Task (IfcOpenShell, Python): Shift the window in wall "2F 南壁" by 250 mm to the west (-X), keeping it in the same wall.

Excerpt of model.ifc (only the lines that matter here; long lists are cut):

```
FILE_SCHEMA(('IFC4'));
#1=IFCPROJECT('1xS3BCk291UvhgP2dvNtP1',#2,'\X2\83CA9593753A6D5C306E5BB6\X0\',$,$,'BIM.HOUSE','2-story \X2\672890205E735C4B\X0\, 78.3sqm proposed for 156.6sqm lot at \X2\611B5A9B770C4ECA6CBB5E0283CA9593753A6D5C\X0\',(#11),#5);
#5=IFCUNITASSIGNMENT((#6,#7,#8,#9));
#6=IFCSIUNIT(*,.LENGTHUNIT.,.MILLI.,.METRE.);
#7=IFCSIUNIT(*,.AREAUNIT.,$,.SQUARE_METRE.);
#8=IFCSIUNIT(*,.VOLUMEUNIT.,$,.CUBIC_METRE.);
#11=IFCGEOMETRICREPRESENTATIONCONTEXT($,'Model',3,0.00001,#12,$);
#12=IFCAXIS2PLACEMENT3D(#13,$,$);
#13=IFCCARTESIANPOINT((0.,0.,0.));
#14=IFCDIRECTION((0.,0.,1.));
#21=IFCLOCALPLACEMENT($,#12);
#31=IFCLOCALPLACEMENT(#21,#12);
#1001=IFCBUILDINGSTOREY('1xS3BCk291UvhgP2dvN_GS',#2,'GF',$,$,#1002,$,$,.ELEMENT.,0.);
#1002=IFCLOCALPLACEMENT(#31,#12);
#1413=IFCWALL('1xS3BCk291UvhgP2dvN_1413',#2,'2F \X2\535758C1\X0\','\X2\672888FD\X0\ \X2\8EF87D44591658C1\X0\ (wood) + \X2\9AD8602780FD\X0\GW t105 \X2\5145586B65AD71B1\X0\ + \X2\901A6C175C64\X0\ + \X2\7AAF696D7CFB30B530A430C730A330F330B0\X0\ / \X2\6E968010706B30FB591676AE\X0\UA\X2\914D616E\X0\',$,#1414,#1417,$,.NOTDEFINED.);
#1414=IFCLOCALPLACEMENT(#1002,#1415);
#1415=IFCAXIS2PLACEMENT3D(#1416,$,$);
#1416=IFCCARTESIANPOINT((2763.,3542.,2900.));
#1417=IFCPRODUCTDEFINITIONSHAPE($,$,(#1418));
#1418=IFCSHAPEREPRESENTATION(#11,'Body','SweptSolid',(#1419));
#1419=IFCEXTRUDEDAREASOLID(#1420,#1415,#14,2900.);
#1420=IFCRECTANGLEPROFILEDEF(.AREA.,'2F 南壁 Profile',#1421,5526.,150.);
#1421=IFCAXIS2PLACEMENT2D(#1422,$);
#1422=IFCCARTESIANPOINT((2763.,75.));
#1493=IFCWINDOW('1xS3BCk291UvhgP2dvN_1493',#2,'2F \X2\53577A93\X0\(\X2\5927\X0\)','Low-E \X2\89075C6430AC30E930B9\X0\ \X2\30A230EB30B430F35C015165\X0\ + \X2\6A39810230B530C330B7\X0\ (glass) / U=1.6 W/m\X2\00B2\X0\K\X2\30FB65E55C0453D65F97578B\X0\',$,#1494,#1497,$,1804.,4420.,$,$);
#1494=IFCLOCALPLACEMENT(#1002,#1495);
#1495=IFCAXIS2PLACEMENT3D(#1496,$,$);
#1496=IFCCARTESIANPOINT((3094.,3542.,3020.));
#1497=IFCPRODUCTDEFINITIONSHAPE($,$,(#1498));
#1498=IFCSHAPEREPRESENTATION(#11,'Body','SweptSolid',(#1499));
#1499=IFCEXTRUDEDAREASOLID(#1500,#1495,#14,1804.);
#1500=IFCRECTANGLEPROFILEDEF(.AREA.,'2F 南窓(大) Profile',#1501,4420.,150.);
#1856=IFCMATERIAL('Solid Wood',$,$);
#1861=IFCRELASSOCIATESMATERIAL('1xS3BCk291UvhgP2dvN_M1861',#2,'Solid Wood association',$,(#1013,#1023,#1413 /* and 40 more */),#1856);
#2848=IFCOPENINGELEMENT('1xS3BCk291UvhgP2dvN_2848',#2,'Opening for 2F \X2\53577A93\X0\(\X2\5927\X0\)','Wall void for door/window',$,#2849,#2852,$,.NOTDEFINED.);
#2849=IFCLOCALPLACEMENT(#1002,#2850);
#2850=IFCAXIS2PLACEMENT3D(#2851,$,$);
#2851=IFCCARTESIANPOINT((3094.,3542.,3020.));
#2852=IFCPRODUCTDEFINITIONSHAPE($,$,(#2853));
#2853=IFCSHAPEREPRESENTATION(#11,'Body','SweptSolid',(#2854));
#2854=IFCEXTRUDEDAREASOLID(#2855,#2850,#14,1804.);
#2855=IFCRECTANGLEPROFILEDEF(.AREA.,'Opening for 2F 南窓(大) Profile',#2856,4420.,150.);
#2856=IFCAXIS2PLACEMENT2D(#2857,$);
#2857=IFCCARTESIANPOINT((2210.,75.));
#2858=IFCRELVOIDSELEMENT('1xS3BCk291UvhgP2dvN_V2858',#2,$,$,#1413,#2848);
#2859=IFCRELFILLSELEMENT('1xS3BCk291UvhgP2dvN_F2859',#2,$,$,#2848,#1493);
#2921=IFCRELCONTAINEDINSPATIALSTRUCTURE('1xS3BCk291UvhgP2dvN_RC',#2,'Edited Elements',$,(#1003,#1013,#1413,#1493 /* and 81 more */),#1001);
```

```python
import ifcopenshell
import ifcopenshell.api.geometry
import ifcopenshell.util.placement
import ifcopenshell.util.unit

model = ifcopenshell.open("model.ifc")
unit_scale = ifcopenshell.util.unit.calculate_unit_scale(model)

window = model.by_guid("1xS3BCk291UvhgP2dvN_1493")
opening = window.FillsVoids[0].RelatingOpeningElement
wall = opening.VoidsElements[0].RelatingBuildingElement

wall_matrix = ifcopenshell.util.placement.get_local_placement(wall.ObjectPlacement)
shift = wall_matrix[:3, 0] * -0.25 / unit_scale
before = ifcopenshell.util.placement.get_local_placement(window.ObjectPlacement)[:3, 3].copy()

# The window is not placed relative to its opening, so move both.
for product in (opening, window):
    matrix = ifcopenshell.util.placement.get_local_placement(product.ObjectPlacement)
    matrix[:3, 3] += shift
    ifcopenshell.api.geometry.edit_object_placement(model, product=product, matrix=matrix, is_si=False)

after = ifcopenshell.util.placement.get_local_placement(window.ObjectPlacement)[:3, 3]
print("window moved by", (after - before).round(3) + 0.0)

model.write("model-out.ifc")
```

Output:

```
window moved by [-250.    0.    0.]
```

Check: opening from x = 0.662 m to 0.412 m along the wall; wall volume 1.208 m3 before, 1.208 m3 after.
